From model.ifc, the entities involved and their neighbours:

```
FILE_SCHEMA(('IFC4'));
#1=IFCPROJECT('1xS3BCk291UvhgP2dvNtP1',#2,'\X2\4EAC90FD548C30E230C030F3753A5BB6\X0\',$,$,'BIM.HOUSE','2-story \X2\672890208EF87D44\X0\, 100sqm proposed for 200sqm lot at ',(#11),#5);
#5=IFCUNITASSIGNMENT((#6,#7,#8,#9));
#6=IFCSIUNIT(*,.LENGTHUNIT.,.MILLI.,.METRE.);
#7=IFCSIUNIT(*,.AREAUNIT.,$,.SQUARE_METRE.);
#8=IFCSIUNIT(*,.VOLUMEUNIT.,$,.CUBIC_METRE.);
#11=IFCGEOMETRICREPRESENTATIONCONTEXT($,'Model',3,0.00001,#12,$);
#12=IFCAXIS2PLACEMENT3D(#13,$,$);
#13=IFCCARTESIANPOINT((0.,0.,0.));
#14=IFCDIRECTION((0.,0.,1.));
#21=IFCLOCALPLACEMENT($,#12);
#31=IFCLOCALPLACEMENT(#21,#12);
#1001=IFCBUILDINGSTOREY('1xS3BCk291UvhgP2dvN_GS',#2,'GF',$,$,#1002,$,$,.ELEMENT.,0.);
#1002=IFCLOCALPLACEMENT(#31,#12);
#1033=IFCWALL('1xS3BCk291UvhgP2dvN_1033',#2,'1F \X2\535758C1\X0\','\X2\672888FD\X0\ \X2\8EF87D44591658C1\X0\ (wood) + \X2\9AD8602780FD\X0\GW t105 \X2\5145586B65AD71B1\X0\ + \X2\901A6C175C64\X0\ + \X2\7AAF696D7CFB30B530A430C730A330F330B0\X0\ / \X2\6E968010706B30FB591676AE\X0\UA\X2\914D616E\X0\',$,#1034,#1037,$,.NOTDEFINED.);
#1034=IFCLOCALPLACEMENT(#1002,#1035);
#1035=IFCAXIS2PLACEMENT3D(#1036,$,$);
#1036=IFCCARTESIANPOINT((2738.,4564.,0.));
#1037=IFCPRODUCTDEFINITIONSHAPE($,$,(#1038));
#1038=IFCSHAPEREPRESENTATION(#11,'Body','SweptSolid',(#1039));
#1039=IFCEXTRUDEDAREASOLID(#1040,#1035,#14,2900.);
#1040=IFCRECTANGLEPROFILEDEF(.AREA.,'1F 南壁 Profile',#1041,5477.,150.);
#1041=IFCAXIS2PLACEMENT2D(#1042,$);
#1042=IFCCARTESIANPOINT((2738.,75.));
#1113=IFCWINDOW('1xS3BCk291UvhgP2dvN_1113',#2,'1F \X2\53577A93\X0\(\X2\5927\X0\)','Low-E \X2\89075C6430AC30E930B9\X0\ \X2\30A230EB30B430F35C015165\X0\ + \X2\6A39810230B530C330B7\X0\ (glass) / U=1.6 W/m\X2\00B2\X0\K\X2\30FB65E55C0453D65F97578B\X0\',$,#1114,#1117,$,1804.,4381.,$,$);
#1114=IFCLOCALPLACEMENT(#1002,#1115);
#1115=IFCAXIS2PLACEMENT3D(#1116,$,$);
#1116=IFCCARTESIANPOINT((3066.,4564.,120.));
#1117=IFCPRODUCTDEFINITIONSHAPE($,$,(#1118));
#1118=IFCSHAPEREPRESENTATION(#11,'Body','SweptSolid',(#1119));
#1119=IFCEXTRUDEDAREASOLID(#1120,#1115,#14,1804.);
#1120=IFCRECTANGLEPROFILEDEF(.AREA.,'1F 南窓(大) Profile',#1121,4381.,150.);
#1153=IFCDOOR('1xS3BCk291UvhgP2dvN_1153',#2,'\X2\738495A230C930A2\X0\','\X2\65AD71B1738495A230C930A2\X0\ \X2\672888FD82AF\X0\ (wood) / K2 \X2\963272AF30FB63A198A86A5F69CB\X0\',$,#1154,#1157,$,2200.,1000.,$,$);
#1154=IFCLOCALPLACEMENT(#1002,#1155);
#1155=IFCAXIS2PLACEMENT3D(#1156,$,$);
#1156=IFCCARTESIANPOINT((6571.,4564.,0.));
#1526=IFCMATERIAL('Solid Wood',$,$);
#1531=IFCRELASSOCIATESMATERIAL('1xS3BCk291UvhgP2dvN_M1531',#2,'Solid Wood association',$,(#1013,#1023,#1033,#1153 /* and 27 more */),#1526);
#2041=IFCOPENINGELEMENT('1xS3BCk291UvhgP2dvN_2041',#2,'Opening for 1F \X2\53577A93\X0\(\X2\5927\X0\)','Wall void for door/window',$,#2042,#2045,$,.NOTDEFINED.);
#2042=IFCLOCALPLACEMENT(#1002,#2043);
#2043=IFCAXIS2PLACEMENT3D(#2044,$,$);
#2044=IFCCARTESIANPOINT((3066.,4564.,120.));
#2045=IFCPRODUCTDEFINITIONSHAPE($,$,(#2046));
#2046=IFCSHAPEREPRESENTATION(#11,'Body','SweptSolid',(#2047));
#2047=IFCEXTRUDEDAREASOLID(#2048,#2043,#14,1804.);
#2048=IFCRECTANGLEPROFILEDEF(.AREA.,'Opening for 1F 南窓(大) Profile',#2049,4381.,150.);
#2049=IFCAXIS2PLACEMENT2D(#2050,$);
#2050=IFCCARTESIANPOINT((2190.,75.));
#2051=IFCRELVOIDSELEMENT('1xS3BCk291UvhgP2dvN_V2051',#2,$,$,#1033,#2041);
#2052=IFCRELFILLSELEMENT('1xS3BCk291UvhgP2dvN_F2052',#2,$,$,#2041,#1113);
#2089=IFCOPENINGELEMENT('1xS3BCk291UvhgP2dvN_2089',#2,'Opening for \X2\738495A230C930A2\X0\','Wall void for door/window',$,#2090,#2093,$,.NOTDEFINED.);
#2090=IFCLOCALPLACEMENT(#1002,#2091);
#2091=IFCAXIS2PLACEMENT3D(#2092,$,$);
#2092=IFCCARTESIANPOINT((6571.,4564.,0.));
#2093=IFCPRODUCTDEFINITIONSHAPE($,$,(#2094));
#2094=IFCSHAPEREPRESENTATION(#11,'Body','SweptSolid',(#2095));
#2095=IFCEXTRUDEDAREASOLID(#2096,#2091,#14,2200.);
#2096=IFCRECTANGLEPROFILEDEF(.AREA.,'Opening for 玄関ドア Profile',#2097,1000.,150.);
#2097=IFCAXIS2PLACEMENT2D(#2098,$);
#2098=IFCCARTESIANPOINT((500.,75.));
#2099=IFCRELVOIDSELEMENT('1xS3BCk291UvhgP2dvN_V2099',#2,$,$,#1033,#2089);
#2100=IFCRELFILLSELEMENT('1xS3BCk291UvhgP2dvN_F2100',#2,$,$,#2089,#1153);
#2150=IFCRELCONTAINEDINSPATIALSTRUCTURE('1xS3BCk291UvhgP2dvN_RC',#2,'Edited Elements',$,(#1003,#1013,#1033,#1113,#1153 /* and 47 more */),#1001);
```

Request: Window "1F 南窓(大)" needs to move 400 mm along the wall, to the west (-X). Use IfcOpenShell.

```python
import ifcopenshell
import ifcopenshell.api.geometry
import ifcopenshell.util.placement

model = ifcopenshell.open("model.ifc")

window = model.by_guid("1xS3BCk291UvhgP2dvN_1113")
opening = window.FillsVoids[0].RelatingOpeningElement
wall = opening.VoidsElements[0].RelatingBuildingElement

wall_matrix = ifcopenshell.util.placement.get_local_placement(wall.ObjectPlacement)
shift = wall_matrix[:3, 0] * -400.0
before = ifcopenshell.util.placement.get_local_placement(window.ObjectPlacement)[:3, 3].copy()

# The window is not placed relative to its opening, so move both.
for product in (opening, window):
    matrix = ifcopenshell.util.placement.get_local_placement(product.ObjectPlacement)
    matrix[:3, 3] += shift
    ifcopenshell.api.geometry.edit_object_placement(model, product=product, matrix=matrix, is_si=False)

after = ifcopenshell.util.placement.get_local_placement(window.ObjectPlacement)[:3, 3]
print("window moved by", (after - before).round(3) + 0.0)

model.write("model_v2.ifc")
```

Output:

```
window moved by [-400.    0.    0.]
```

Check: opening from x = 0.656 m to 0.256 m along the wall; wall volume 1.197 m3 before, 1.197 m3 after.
